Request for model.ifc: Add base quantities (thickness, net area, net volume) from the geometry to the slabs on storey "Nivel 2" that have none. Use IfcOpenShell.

First a look at what the model holds.

```python
import ifcopenshell
import ifcopenshell.util.element
import ifcopenshell.util.unit

model = ifcopenshell.open("model.ifc")
print(model.schema)
for unit_type in ("LENGTHUNIT", "AREAUNIT", "VOLUMEUNIT"):
    print(unit_type, ifcopenshell.util.unit.calculate_unit_scale(model, unit_type))
storey = next(s for s in model.by_type("IfcBuildingStorey") if s.Name == "Nivel 2")
slabs = [e for e in ifcopenshell.util.element.get_decomposition(storey) if e.is_a("IfcSlab")]
for e in sorted(slabs, key=lambda e: e.id()):
    print(e.id(), e.is_a(), e.Name, list(ifcopenshell.util.element.get_psets(e, qtos_only=True)), sep=" | ")
```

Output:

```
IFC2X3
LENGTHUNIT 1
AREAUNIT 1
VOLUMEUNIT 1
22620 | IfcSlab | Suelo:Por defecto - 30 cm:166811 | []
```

```python
import ifcopenshell
import ifcopenshell.api.pset
import ifcopenshell.geom
import ifcopenshell.util.element
import ifcopenshell.util.shape
import ifcopenshell.util.unit

model = ifcopenshell.open("model.ifc")
unit_scale = ifcopenshell.util.unit.calculate_unit_scale(model)
area_scale = ifcopenshell.util.unit.calculate_unit_scale(model, "AREAUNIT")
volume_scale = ifcopenshell.util.unit.calculate_unit_scale(model, "VOLUMEUNIT")
settings = ifcopenshell.geom.settings()

storey = next(s for s in model.by_type("IfcBuildingStorey") if s.Name == "Nivel 2")
slabs = [e for e in ifcopenshell.util.element.get_decomposition(storey) if e.is_a("IfcSlab")]

for e in sorted(slabs, key=lambda e: e.id()):
    if ifcopenshell.util.element.get_psets(e, qtos_only=True, should_inherit=False):
        continue
    # Geometry comes back in metres, in the element's own axes.
    shape = ifcopenshell.geom.create_shape(settings, e)
    values = {
        "Width": ifcopenshell.util.shape.get_z(shape.geometry) / unit_scale,
        "NetArea": ifcopenshell.util.shape.get_footprint_area(shape.geometry) / area_scale,
        "NetVolume": ifcopenshell.util.shape.get_volume(shape.geometry) / volume_scale,
    }
    qto = ifcopenshell.api.pset.add_qto(model, product=e, name="BaseQuantities")
    ifcopenshell.api.pset.edit_qto(model, qto=qto, properties=values)
    print(e.id(), {k: round(v, 3) for k, v in values.items()})

model.write("model_updated.ifc")
```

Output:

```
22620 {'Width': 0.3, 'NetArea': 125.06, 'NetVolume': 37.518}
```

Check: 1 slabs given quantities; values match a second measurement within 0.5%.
